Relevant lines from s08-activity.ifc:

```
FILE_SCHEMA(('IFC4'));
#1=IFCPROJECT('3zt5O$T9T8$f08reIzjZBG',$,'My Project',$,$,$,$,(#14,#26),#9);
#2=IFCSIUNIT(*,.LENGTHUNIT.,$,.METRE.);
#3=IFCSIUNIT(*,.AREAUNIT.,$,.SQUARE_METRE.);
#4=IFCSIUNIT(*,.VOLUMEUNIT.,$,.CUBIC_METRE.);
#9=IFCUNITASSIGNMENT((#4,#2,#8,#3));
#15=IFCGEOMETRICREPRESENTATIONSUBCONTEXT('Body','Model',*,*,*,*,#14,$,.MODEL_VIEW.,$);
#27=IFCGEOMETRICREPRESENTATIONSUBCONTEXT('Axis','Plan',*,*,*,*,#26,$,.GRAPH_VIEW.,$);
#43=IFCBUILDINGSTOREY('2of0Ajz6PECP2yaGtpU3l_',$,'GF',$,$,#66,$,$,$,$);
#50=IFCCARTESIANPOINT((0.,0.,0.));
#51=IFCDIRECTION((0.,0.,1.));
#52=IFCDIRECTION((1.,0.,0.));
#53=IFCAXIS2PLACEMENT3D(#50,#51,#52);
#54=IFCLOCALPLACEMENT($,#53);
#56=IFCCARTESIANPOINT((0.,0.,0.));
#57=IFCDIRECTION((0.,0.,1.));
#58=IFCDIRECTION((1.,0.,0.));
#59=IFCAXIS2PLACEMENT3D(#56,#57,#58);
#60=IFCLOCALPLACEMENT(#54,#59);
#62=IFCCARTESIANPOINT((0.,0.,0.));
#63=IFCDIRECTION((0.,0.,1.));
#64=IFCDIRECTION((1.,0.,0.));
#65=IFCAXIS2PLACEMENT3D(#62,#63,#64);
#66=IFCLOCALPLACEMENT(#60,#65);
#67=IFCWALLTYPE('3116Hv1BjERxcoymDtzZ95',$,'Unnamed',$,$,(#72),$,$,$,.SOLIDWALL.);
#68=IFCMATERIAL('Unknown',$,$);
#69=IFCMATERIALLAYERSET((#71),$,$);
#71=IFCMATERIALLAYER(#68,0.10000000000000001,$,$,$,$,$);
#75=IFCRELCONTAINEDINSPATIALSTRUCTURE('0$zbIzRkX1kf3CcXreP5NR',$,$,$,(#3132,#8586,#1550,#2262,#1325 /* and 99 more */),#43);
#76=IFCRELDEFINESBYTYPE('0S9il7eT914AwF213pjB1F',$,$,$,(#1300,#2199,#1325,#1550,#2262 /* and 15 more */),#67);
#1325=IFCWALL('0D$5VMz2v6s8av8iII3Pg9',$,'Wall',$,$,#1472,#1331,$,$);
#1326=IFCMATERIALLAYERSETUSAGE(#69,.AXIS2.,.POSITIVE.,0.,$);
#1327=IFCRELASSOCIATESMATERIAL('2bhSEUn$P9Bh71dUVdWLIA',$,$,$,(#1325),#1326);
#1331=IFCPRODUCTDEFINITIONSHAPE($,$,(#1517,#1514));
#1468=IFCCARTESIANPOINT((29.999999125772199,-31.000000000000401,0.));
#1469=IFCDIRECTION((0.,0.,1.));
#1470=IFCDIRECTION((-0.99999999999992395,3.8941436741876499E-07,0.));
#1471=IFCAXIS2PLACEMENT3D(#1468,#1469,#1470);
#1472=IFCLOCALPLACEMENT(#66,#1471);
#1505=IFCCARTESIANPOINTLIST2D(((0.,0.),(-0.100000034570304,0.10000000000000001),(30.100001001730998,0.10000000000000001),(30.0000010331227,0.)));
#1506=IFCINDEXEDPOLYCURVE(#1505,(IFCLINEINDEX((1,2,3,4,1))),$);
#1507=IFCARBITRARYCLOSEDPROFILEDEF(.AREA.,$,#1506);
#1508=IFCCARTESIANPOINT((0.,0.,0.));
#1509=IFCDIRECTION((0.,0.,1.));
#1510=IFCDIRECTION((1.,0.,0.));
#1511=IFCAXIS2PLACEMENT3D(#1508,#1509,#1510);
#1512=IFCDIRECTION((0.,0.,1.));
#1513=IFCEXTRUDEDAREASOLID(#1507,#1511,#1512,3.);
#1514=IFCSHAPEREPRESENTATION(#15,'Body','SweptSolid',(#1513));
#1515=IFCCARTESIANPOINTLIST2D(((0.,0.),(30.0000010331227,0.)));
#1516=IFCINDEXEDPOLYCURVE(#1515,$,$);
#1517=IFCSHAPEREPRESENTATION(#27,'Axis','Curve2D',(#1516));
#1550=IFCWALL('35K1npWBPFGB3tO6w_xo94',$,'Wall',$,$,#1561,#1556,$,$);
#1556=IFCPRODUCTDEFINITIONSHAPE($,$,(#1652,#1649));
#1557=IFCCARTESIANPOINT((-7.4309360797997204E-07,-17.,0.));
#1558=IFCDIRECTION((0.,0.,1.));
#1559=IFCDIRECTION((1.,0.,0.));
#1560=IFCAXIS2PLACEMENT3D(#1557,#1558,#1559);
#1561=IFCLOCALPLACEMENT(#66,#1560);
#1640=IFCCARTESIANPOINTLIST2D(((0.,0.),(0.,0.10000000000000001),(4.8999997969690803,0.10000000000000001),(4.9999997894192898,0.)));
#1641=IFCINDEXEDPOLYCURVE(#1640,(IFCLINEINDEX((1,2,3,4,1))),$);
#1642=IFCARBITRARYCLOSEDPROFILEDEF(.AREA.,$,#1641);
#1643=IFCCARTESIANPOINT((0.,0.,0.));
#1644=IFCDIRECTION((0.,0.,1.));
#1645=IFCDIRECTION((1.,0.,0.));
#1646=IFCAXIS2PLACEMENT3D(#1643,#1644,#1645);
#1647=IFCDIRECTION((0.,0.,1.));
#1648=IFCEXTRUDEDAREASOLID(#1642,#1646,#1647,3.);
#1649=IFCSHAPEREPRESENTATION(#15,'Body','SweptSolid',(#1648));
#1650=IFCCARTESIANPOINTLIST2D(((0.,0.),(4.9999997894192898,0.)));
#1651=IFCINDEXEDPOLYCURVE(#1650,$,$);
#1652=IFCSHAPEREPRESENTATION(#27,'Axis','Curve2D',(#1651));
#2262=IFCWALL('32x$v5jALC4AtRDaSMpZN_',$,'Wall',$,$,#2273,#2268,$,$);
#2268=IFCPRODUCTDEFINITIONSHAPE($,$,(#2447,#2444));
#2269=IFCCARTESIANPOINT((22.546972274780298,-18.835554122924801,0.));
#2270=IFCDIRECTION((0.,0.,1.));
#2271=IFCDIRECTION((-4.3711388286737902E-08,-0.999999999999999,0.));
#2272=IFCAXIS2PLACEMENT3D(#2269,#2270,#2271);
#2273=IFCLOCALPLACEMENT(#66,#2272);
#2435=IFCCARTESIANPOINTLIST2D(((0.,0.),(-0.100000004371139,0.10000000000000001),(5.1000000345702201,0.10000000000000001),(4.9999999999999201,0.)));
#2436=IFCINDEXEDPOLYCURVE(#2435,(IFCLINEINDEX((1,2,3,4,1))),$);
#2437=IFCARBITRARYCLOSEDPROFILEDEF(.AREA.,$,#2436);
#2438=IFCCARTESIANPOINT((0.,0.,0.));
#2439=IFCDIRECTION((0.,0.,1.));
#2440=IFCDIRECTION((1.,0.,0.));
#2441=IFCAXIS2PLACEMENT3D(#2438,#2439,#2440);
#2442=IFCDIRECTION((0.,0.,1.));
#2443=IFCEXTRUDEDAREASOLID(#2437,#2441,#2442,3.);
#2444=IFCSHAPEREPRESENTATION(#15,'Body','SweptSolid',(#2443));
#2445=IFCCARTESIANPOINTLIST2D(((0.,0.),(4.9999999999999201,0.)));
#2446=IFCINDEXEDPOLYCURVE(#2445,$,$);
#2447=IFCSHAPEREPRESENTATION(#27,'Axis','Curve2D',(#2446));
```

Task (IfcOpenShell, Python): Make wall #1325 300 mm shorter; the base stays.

```python
import ifcopenshell
import ifcopenshell.geom
import ifcopenshell.util.representation
import ifcopenshell.util.shape

model = ifcopenshell.open("s08-activity.ifc")
settings = ifcopenshell.geom.settings()


def volume(element):
    """Net volume in cubic metres, openings subtracted."""
    shape = ifcopenshell.geom.create_shape(settings, element)
    return ifcopenshell.util.shape.get_volume(shape.geometry)


wall = model.by_guid("0D$5VMz2v6s8av8iII3Pg9")
before = volume(wall)

body = ifcopenshell.util.representation.get_representation(wall, "Model", "Body")
solid = body.Items[0]
old_height = solid.Depth
solid.Depth -= 0.3
after = volume(wall)

print(f"height {old_height:g} -> {solid.Depth:g}, volume {before:.3f} -> {after:.3f} m3")

model.write("s08-activity_edited.ifc")
```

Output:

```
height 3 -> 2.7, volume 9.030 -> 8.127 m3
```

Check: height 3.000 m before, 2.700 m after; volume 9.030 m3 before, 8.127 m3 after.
